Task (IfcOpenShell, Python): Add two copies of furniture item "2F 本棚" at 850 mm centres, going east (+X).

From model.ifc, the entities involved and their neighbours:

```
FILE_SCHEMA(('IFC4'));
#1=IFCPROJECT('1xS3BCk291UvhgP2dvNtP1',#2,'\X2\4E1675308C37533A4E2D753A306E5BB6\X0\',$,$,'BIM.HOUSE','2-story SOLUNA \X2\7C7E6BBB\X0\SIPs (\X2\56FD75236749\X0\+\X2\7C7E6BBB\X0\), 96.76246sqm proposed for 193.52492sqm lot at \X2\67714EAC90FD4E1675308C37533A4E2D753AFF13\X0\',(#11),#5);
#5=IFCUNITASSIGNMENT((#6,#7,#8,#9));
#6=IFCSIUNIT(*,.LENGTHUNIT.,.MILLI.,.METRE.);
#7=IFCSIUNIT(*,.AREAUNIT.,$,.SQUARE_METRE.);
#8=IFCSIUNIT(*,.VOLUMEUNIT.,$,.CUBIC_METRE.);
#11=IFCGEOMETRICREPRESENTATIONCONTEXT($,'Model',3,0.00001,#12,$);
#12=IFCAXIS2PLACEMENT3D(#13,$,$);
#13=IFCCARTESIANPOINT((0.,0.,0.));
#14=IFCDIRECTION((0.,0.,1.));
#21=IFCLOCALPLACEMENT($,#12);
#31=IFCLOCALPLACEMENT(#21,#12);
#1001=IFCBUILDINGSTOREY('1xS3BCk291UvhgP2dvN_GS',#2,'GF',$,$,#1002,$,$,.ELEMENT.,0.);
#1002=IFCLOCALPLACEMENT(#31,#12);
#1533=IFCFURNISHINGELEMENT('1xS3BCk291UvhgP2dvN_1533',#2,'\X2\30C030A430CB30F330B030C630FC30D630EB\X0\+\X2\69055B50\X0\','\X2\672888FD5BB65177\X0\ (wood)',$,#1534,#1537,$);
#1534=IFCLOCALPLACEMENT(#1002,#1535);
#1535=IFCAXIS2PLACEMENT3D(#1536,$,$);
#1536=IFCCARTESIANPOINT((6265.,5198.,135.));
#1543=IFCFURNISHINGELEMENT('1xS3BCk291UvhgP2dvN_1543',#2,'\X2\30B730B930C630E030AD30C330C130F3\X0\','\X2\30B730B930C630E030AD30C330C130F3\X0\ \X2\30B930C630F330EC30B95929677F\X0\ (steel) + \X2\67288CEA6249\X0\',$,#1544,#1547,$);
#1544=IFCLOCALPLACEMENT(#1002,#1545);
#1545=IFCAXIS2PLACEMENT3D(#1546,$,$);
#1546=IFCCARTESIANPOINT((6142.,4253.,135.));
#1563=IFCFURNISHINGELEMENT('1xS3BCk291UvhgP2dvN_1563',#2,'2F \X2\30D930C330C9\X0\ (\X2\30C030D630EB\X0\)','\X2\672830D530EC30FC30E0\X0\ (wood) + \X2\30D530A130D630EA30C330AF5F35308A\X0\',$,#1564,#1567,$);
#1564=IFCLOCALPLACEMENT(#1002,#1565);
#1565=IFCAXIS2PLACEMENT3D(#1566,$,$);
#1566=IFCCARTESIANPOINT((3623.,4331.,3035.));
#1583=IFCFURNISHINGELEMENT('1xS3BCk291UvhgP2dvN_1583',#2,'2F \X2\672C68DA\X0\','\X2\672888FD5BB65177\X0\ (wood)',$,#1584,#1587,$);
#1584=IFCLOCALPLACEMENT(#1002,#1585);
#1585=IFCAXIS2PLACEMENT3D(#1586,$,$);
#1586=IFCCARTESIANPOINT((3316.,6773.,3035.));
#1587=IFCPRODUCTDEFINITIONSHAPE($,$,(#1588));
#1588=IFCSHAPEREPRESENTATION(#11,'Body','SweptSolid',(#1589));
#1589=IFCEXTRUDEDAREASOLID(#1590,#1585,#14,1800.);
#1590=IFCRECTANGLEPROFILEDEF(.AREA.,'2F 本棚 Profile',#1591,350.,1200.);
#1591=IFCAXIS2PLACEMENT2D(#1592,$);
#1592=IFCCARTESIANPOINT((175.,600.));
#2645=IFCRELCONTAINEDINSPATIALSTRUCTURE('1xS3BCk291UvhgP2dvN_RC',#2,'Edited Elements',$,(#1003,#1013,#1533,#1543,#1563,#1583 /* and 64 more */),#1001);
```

```python
import numpy as np
import ifcopenshell
import ifcopenshell.api.geometry
import ifcopenshell.api.root
import ifcopenshell.util.element
import ifcopenshell.util.placement
import ifcopenshell.util.unit

model = ifcopenshell.open("model.ifc")
unit_scale = ifcopenshell.util.unit.calculate_unit_scale(model)


def reuse_history(source, copy):
    """copy_class also copies each property set's owner history, people and application; keep the originals."""
    for rel in copy.IsDefinedBy:
        if rel.is_a("IfcRelDefinesByProperties") and (history := rel.RelatingPropertyDefinition.OwnerHistory):
            rel.RelatingPropertyDefinition.OwnerHistory = source.OwnerHistory
            ifcopenshell.util.element.remove_deep2(model, history)


source = model.by_guid("1xS3BCk291UvhgP2dvN_1583")
base = ifcopenshell.util.placement.get_local_placement(source.ObjectPlacement)
step = np.array([1.0, 0.0, 0.0]) * 0.85 / unit_scale

for i in range(1, 3):
    copy = ifcopenshell.api.root.copy_class(model, product=source)
    copy.Representation = ifcopenshell.util.element.copy_deep(
        model, source.Representation, exclude=["IfcGeometricRepresentationContext", "IfcRepresentationMap"]
    )
    reuse_history(source, copy)
    matrix = base.copy()
    matrix[:3, 3] += i * step
    print("added at", matrix[:3, 3].round(3) + 0.0)
    ifcopenshell.api.geometry.edit_object_placement(model, product=copy, matrix=matrix, is_si=False)

model.write("model_rev.ifc")
```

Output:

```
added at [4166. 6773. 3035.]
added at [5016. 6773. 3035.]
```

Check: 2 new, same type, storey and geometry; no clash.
